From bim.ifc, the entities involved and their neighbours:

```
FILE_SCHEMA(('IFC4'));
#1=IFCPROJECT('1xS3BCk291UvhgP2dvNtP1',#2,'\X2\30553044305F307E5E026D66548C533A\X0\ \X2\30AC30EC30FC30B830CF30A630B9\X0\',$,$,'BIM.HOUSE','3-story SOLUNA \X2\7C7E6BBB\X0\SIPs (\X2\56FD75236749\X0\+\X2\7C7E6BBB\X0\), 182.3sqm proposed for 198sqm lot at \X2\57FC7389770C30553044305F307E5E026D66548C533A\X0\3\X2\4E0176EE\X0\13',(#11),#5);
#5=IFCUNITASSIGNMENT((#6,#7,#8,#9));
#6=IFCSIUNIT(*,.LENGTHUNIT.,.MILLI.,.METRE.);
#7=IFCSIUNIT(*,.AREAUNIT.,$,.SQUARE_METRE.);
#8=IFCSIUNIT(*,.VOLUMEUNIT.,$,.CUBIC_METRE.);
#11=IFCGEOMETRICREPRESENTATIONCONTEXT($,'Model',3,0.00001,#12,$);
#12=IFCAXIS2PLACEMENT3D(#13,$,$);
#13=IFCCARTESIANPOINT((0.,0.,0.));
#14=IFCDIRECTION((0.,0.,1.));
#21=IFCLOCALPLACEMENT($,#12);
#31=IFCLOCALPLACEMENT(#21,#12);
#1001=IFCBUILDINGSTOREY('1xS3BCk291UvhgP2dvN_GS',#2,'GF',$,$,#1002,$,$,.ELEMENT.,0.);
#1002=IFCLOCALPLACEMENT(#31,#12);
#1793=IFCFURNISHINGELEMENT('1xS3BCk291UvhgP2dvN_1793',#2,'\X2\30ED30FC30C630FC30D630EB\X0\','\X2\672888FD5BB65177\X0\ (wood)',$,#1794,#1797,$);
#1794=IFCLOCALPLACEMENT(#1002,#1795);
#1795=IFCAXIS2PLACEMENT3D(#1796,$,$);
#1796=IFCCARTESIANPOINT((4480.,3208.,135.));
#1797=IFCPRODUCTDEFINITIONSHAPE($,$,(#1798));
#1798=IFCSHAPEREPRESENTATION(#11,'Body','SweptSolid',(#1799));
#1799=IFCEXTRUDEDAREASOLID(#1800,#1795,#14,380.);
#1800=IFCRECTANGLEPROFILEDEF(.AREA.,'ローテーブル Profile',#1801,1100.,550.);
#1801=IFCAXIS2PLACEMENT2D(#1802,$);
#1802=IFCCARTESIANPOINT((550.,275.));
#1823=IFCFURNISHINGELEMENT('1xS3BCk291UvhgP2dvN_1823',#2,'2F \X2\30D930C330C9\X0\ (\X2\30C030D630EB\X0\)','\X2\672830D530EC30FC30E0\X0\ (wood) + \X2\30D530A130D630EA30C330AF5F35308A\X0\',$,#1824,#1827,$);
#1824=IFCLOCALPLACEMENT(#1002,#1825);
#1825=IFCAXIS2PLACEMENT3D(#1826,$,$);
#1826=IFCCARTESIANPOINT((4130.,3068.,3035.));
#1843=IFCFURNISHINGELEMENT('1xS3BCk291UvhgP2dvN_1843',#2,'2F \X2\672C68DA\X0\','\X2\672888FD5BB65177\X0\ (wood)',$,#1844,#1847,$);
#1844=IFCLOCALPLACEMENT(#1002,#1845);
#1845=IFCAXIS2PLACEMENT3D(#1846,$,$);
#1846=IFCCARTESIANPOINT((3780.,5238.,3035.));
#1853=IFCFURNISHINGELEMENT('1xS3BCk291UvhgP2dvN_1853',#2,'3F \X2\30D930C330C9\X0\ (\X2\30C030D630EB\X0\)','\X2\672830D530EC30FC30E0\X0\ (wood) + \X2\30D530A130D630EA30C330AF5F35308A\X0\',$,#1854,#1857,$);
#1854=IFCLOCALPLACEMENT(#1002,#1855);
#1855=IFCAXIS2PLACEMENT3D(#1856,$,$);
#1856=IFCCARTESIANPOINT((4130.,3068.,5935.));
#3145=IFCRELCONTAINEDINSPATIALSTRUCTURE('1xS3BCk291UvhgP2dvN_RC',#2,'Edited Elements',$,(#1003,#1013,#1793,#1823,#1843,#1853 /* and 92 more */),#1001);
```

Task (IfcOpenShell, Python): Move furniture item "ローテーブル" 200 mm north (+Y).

```python
import ifcopenshell
import ifcopenshell.api.geometry
import ifcopenshell.util.placement
import ifcopenshell.util.unit

model = ifcopenshell.open("bim.ifc")
unit_scale = ifcopenshell.util.unit.calculate_unit_scale(model)

item = model.by_guid("1xS3BCk291UvhgP2dvN_1793")
matrix = ifcopenshell.util.placement.get_local_placement(item.ObjectPlacement)
matrix[1, 3] += 0.2 / unit_scale
ifcopenshell.api.geometry.edit_object_placement(model, product=item, matrix=matrix, is_si=False)

print(ifcopenshell.util.placement.get_local_placement(item.ObjectPlacement).round(3) + 0.0)

model.write("bim_rev.ifc")
```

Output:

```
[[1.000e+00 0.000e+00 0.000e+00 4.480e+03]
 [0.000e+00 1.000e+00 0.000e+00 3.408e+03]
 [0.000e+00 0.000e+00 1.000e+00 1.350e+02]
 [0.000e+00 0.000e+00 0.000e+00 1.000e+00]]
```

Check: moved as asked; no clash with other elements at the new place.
